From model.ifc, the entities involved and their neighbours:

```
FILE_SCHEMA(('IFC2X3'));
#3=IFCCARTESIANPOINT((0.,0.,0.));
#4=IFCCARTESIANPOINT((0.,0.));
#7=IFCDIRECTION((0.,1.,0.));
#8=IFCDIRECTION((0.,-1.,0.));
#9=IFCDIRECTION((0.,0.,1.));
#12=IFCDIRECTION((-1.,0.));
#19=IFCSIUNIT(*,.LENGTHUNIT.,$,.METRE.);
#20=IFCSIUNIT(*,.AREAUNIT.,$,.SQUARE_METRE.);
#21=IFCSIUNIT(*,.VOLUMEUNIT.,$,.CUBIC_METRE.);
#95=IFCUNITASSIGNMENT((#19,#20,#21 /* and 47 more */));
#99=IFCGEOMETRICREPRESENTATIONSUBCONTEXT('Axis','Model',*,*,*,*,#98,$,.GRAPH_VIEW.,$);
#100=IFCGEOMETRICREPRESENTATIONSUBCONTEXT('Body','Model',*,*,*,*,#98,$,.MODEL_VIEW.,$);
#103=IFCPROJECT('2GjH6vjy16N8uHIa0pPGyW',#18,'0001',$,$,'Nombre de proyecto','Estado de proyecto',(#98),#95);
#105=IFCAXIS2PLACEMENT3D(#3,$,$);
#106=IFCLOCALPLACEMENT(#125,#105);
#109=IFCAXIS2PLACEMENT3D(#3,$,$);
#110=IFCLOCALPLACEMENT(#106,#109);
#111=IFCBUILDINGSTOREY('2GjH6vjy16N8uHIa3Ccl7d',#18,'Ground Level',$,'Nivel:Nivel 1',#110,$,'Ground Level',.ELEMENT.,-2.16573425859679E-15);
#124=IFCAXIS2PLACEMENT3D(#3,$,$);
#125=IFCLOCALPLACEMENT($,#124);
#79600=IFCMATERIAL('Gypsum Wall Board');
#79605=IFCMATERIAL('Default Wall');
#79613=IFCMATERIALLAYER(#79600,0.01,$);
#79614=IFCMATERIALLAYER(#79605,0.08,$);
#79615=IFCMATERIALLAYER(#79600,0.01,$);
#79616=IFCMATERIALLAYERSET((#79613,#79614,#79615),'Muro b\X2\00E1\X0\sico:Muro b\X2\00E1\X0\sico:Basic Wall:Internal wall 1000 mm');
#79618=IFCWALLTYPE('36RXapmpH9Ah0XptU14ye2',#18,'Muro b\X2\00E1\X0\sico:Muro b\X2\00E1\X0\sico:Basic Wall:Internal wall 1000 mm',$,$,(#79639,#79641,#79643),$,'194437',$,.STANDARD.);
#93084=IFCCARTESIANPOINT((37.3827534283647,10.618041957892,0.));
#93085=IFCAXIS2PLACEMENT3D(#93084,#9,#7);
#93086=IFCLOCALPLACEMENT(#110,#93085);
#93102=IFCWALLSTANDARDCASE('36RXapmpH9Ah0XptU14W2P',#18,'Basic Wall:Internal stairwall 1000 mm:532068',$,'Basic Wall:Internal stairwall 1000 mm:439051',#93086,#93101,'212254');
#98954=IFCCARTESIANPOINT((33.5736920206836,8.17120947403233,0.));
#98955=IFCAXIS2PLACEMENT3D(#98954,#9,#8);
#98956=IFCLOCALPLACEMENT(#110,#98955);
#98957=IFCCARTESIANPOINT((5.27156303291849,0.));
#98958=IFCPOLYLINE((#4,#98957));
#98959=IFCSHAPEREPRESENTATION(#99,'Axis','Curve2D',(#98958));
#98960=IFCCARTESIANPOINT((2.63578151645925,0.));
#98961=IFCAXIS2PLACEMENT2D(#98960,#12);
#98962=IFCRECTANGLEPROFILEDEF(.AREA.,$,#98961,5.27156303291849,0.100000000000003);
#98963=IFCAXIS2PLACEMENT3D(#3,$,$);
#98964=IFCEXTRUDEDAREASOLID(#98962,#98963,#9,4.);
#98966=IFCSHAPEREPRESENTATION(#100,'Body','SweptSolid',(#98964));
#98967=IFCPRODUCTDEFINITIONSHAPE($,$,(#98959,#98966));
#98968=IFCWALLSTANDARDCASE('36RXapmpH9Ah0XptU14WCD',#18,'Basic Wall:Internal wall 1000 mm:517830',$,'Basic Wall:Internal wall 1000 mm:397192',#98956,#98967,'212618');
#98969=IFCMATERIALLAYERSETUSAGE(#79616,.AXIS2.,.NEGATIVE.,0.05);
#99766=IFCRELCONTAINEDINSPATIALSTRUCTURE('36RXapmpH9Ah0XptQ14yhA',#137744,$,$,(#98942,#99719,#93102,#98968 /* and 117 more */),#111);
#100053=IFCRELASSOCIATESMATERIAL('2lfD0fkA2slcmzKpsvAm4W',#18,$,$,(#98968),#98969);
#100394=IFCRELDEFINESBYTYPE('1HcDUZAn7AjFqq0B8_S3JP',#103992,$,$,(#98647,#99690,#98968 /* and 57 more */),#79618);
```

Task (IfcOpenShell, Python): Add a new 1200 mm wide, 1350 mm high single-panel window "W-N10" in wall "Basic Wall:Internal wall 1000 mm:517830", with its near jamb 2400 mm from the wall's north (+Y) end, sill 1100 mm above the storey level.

```python
import numpy as np
import ifcopenshell
import ifcopenshell.api.feature
import ifcopenshell.api.geometry
import ifcopenshell.api.root
import ifcopenshell.api.spatial
import ifcopenshell.api.type
import ifcopenshell.geom
import ifcopenshell.util.element
import ifcopenshell.util.placement
import ifcopenshell.util.representation
import ifcopenshell.util.shape
import ifcopenshell.util.unit

model = ifcopenshell.open("model.ifc")
unit_scale = ifcopenshell.util.unit.calculate_unit_scale(model)
settings = ifcopenshell.geom.settings()


def volume(element):
    """Net volume in cubic metres, openings subtracted."""
    shape = ifcopenshell.geom.create_shape(settings, element)
    return ifcopenshell.util.shape.get_volume(shape.geometry)


wall = model.by_guid("36RXapmpH9Ah0XptU14WCD")
storey = ifcopenshell.util.element.get_container(wall, ifc_class="IfcBuildingStorey")
context = ifcopenshell.util.representation.get_context(model, "Model", "Body", "MODEL_VIEW")
before = volume(wall)

width, height, from_end, sill = 1.2, 1.35, 2.4, 1.1  # metres

# The wall runs along its own X axis, and the end named is its -X end.
wall_shape = ifcopenshell.geom.create_shape(settings, wall)
x, y, z = ifcopenshell.util.shape.get_vertices(wall_shape.geometry).T
start = x.min() + from_end
face, thickness = float(y.min()), float(y.max() - y.min())
wall_matrix = ifcopenshell.util.placement.get_local_placement(wall.ObjectPlacement)
level = ifcopenshell.util.placement.get_local_placement(storey.ObjectPlacement)[2, 3]


def in_wall(x, y):
    """Placement at x, y metres in the wall's axes, at sill height."""
    matrix = wall_matrix.copy()
    matrix[:, 3] = wall_matrix @ np.array([x / unit_scale, y / unit_scale, 0.0, 1.0])
    matrix[2, 3] = level + sill / unit_scale
    return matrix


# Opening: a box that overshoots both wall faces by 50 mm.
opening = ifcopenshell.api.root.create_entity(model, ifc_class="IfcOpeningElement")
box = ifcopenshell.api.geometry.add_wall_representation(
    model, context=context, length=width, height=height, thickness=thickness + 0.1
)
ifcopenshell.api.geometry.assign_representation(model, product=opening, representation=box)
ifcopenshell.api.geometry.edit_object_placement(model, product=opening, matrix=in_wall(start, face - 0.05), is_si=False)
ifcopenshell.api.feature.add_feature(model, feature=opening, element=wall)

window = ifcopenshell.api.root.create_entity(model, ifc_class="IfcWindow", name="W-N10")
window.OverallWidth, window.OverallHeight = width / unit_scale, height / unit_scale
body = ifcopenshell.api.geometry.add_window_representation(
    model,
    context=context,
    overall_width=window.OverallWidth,
    overall_height=window.OverallHeight,
    partition_type="SINGLE_PANEL",
)
ifcopenshell.api.geometry.assign_representation(model, product=window, representation=body)
ifcopenshell.api.spatial.assign_container(model, products=[window], relating_structure=storey)
fills = ifcopenshell.api.feature.add_filling(model, opening=opening, element=window)
fills.OwnerHistory = window.OwnerHistory  # required in IFC2X3

# IFC2X3 keeps the operation on the window style.
style = ifcopenshell.api.root.create_entity(model, ifc_class="IfcWindowStyle", name="W-N10")
style.OperationType, style.ConstructionType = "SINGLE_PANEL", "NOTDEFINED"
style.ParameterTakesPrecedence = style.Sizeable = False
ifcopenshell.api.type.assign_type(model, related_objects=[window], relating_type=style)

# Centre the window in the wall's thickness.
ifcopenshell.api.geometry.edit_object_placement(model, product=window, matrix=in_wall(start, face), is_si=False)
window_shape = ifcopenshell.geom.create_shape(settings, window)
depth = ifcopenshell.util.shape.get_vertices(window_shape.geometry)[:, 1]
offset = face + thickness / 2 - (depth.min() + depth.max()) / 2
ifcopenshell.api.geometry.edit_object_placement(model, product=window, matrix=in_wall(start, offset), is_si=False)

after = volume(wall)

print(f"wall volume {before:.3f} -> {after:.3f} m3")

model.write("model_v2.ifc")
```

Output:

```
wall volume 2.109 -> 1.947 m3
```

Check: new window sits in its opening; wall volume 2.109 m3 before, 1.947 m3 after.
